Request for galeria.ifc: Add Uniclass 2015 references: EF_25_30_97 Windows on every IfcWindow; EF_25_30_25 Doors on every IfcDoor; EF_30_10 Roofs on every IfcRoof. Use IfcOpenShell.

First a look at what the model holds.

```python
import ifcopenshell

model = ifcopenshell.open("galeria.ifc")
print(model.schema)
print("classifications:", [c.Name for c in model.by_type("IfcClassification")])
for ifc_class in ("IfcDoor", "IfcRoof", "IfcStair", "IfcWall", "IfcWindow"):
    print(ifc_class, len(model.by_type(ifc_class)))
```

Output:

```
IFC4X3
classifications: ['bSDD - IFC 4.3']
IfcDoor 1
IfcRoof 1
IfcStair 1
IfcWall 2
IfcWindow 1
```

```python
import ifcopenshell
import ifcopenshell.api.classification

model = ifcopenshell.open("galeria.ifc")

system = ifcopenshell.api.classification.add_classification(model, classification="Uniclass 2015")

codes = {
    "IfcWindow": ("EF_25_30_97", "Windows"),
    "IfcDoor": ("EF_25_30_25", "Doors"),
    "IfcRoof": ("EF_30_10", "Roofs"),
}
for ifc_class, (code, name) in codes.items():
    products = model.by_type(ifc_class)
    ifcopenshell.api.classification.add_reference(
        model, products=products, classification=system, identification=code, name=name
    )
    print(code, len(products))

model.write("galeria_v2.ifc")
```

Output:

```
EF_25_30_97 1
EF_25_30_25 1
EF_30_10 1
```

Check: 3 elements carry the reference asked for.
